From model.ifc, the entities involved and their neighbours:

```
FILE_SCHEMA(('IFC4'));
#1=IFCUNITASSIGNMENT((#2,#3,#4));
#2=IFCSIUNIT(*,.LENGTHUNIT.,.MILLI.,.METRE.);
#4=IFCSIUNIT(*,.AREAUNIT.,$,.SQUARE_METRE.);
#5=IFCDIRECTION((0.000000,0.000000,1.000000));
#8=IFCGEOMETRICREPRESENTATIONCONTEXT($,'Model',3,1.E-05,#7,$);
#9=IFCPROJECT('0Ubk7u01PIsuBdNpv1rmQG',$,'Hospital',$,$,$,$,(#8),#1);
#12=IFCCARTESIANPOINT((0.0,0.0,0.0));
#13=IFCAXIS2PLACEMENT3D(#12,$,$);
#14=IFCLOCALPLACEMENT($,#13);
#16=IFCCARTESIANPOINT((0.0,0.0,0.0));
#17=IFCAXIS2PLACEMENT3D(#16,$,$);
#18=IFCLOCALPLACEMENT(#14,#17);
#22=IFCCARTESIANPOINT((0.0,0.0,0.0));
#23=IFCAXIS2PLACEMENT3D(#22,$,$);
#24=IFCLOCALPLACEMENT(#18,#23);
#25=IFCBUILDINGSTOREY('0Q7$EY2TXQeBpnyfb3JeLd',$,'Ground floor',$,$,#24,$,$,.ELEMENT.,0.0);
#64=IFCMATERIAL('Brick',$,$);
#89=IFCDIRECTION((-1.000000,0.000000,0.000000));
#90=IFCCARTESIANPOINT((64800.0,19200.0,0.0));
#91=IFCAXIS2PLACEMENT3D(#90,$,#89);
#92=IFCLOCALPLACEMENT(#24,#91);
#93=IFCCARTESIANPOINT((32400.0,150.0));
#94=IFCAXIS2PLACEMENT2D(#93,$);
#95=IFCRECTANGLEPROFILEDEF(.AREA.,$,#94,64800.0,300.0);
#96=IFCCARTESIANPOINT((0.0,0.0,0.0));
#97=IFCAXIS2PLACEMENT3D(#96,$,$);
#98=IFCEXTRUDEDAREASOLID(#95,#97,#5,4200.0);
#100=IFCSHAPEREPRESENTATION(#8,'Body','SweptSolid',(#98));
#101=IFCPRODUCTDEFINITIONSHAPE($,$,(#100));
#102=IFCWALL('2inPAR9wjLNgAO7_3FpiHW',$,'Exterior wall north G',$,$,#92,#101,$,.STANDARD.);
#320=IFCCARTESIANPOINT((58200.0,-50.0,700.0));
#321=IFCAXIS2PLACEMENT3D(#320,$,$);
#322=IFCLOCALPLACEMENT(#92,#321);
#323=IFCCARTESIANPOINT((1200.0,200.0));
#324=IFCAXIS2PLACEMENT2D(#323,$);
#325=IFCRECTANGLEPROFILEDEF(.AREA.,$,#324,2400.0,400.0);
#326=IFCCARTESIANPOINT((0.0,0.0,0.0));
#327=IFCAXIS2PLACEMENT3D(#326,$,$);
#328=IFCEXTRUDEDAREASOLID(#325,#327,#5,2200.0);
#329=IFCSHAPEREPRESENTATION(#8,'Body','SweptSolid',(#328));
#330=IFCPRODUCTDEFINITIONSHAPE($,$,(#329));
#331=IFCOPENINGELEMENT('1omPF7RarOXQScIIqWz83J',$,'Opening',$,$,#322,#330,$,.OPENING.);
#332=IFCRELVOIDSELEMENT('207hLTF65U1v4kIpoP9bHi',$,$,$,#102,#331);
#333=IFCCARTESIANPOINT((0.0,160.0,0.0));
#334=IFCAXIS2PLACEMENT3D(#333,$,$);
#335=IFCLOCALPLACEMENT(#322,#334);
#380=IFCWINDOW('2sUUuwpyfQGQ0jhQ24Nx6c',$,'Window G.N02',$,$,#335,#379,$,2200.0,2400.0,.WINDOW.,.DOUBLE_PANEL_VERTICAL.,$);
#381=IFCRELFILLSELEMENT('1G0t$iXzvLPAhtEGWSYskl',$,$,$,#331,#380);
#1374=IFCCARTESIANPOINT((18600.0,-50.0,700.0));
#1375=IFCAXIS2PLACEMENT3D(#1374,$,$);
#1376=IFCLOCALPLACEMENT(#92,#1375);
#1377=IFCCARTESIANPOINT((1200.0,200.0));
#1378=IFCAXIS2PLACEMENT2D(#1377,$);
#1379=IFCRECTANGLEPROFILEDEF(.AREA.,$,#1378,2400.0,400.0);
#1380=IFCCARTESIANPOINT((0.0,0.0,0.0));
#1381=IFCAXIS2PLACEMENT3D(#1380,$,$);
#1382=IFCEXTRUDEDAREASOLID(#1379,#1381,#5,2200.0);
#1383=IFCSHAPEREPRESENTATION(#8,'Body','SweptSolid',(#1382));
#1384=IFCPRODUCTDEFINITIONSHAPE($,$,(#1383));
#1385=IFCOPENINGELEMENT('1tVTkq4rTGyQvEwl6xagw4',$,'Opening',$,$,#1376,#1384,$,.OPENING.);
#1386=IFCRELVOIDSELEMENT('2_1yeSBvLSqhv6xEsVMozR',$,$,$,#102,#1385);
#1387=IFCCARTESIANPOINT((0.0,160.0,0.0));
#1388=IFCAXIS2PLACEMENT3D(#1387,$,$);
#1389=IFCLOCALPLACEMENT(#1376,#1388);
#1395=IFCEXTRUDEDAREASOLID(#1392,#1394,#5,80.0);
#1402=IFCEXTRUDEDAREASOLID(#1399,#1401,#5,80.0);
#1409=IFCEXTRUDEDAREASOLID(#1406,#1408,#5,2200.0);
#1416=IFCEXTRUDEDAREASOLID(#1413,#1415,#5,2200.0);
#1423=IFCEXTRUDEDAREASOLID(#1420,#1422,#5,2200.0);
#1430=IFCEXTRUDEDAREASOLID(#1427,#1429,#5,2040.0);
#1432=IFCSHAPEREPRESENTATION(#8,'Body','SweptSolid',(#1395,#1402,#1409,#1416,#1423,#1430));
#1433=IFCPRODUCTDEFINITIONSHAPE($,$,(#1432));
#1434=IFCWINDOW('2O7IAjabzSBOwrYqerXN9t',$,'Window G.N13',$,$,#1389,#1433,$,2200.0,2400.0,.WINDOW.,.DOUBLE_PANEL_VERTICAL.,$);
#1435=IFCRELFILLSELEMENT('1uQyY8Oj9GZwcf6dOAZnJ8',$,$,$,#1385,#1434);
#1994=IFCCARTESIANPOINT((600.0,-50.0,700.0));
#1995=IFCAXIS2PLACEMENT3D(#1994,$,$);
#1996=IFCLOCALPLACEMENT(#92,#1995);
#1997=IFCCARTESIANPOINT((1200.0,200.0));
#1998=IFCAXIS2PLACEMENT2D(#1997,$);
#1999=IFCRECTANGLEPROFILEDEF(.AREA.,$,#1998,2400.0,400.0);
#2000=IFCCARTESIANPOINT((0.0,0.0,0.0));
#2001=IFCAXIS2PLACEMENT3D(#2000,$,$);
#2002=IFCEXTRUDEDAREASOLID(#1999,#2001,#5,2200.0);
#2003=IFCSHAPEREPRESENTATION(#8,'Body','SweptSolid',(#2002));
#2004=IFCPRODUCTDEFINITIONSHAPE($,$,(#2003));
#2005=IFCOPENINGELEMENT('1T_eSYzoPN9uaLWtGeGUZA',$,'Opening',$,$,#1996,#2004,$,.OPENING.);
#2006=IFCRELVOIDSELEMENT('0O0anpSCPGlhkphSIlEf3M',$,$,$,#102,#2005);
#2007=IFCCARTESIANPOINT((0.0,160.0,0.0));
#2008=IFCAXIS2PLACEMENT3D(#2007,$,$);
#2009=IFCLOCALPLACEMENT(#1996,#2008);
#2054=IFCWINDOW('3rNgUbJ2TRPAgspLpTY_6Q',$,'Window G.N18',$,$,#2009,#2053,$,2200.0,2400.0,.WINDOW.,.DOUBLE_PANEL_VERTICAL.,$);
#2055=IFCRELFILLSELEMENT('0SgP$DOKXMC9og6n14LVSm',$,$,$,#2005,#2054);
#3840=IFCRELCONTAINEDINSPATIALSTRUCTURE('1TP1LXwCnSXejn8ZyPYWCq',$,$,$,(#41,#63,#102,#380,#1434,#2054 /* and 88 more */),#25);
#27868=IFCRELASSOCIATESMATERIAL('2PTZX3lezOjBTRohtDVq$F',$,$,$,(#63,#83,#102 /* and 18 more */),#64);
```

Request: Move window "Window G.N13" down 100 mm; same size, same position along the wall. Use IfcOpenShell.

```python
import numpy as np
import ifcopenshell
import ifcopenshell.api.geometry
import ifcopenshell.util.placement
import ifcopenshell.util.unit

model = ifcopenshell.open("model.ifc")
unit_scale = ifcopenshell.util.unit.calculate_unit_scale(model)

window = model.by_guid("2O7IAjabzSBOwrYqerXN9t")
opening = window.FillsVoids[0].RelatingOpeningElement
dz = -100.0

shift = np.array([0.0, 0.0, dz])
# The window is placed relative to its opening, so it follows when the opening moves.
matrix = ifcopenshell.util.placement.get_local_placement(opening.ObjectPlacement)
matrix[:3, 3] += shift
ifcopenshell.api.geometry.edit_object_placement(
    model, product=opening, matrix=matrix, is_si=False, should_transform_children=True
)

print(f"moved by {dz * unit_scale:+.3f} m")

model.write("model_v2.ifc")
```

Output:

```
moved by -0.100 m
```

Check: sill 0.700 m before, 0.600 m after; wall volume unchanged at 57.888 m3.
